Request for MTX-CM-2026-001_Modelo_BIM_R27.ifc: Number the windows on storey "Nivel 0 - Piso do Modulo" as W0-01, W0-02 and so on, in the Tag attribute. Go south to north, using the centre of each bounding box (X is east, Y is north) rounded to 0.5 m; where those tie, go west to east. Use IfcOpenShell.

First a look at what the model holds.

```python
import ifcopenshell
import ifcopenshell.util.element
import ifcopenshell.util.placement

model = ifcopenshell.open("MTX-CM-2026-001_Modelo_BIM_R27.ifc")
print(model.schema)
storey = next(s for s in model.by_type("IfcBuildingStorey") if s.Name == "Nivel 0 - Piso do Modulo")
windows = [e for e in ifcopenshell.util.element.get_decomposition(storey) if e.is_a("IfcWindow")]
for e in sorted(windows, key=lambda e: e.id()):
    origin = ifcopenshell.util.placement.get_local_placement(e.ObjectPlacement)[:3, 3]
    print(e.id(), e.Tag, e.Name, origin.round(2) + 0.0, sep=" | ")
```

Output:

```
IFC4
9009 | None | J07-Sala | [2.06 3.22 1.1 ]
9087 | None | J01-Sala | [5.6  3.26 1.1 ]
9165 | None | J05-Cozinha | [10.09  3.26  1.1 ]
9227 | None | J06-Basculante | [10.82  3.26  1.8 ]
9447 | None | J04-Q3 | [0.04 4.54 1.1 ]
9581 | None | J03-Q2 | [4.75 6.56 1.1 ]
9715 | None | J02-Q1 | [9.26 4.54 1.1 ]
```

```python
import ifcopenshell
import ifcopenshell.geom
import ifcopenshell.util.element
import ifcopenshell.util.shape

model = ifcopenshell.open("MTX-CM-2026-001_Modelo_BIM_R27.ifc")
settings = ifcopenshell.geom.settings()
settings.set("use-world-coords", True)


def centre(element):
    shape = ifcopenshell.geom.create_shape(settings, element)
    return ifcopenshell.util.shape.get_bbox_centroid(shape.geometry)


storey = next(s for s in model.by_type("IfcBuildingStorey") if s.Name == "Nivel 0 - Piso do Modulo")
windows = [e for e in ifcopenshell.util.element.get_decomposition(storey) if e.is_a("IfcWindow")]

# Insertion points can sit at a corner or the storey origin, so sort by the geometry (in metres).
centres = {e: centre(e) for e in windows}
windows.sort(key=lambda e: (round(centres[e][1] / 0.5), centres[e][0]))

for i, e in enumerate(windows, start=1):
    number = f"W0-{i:02d}"
    e.Tag = number
    print(e.id(), number)

model.write("MTX-CM-2026-001_Modelo_BIM_R27-out.ifc")
```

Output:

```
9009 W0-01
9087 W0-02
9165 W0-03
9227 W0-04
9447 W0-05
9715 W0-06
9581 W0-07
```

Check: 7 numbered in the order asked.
